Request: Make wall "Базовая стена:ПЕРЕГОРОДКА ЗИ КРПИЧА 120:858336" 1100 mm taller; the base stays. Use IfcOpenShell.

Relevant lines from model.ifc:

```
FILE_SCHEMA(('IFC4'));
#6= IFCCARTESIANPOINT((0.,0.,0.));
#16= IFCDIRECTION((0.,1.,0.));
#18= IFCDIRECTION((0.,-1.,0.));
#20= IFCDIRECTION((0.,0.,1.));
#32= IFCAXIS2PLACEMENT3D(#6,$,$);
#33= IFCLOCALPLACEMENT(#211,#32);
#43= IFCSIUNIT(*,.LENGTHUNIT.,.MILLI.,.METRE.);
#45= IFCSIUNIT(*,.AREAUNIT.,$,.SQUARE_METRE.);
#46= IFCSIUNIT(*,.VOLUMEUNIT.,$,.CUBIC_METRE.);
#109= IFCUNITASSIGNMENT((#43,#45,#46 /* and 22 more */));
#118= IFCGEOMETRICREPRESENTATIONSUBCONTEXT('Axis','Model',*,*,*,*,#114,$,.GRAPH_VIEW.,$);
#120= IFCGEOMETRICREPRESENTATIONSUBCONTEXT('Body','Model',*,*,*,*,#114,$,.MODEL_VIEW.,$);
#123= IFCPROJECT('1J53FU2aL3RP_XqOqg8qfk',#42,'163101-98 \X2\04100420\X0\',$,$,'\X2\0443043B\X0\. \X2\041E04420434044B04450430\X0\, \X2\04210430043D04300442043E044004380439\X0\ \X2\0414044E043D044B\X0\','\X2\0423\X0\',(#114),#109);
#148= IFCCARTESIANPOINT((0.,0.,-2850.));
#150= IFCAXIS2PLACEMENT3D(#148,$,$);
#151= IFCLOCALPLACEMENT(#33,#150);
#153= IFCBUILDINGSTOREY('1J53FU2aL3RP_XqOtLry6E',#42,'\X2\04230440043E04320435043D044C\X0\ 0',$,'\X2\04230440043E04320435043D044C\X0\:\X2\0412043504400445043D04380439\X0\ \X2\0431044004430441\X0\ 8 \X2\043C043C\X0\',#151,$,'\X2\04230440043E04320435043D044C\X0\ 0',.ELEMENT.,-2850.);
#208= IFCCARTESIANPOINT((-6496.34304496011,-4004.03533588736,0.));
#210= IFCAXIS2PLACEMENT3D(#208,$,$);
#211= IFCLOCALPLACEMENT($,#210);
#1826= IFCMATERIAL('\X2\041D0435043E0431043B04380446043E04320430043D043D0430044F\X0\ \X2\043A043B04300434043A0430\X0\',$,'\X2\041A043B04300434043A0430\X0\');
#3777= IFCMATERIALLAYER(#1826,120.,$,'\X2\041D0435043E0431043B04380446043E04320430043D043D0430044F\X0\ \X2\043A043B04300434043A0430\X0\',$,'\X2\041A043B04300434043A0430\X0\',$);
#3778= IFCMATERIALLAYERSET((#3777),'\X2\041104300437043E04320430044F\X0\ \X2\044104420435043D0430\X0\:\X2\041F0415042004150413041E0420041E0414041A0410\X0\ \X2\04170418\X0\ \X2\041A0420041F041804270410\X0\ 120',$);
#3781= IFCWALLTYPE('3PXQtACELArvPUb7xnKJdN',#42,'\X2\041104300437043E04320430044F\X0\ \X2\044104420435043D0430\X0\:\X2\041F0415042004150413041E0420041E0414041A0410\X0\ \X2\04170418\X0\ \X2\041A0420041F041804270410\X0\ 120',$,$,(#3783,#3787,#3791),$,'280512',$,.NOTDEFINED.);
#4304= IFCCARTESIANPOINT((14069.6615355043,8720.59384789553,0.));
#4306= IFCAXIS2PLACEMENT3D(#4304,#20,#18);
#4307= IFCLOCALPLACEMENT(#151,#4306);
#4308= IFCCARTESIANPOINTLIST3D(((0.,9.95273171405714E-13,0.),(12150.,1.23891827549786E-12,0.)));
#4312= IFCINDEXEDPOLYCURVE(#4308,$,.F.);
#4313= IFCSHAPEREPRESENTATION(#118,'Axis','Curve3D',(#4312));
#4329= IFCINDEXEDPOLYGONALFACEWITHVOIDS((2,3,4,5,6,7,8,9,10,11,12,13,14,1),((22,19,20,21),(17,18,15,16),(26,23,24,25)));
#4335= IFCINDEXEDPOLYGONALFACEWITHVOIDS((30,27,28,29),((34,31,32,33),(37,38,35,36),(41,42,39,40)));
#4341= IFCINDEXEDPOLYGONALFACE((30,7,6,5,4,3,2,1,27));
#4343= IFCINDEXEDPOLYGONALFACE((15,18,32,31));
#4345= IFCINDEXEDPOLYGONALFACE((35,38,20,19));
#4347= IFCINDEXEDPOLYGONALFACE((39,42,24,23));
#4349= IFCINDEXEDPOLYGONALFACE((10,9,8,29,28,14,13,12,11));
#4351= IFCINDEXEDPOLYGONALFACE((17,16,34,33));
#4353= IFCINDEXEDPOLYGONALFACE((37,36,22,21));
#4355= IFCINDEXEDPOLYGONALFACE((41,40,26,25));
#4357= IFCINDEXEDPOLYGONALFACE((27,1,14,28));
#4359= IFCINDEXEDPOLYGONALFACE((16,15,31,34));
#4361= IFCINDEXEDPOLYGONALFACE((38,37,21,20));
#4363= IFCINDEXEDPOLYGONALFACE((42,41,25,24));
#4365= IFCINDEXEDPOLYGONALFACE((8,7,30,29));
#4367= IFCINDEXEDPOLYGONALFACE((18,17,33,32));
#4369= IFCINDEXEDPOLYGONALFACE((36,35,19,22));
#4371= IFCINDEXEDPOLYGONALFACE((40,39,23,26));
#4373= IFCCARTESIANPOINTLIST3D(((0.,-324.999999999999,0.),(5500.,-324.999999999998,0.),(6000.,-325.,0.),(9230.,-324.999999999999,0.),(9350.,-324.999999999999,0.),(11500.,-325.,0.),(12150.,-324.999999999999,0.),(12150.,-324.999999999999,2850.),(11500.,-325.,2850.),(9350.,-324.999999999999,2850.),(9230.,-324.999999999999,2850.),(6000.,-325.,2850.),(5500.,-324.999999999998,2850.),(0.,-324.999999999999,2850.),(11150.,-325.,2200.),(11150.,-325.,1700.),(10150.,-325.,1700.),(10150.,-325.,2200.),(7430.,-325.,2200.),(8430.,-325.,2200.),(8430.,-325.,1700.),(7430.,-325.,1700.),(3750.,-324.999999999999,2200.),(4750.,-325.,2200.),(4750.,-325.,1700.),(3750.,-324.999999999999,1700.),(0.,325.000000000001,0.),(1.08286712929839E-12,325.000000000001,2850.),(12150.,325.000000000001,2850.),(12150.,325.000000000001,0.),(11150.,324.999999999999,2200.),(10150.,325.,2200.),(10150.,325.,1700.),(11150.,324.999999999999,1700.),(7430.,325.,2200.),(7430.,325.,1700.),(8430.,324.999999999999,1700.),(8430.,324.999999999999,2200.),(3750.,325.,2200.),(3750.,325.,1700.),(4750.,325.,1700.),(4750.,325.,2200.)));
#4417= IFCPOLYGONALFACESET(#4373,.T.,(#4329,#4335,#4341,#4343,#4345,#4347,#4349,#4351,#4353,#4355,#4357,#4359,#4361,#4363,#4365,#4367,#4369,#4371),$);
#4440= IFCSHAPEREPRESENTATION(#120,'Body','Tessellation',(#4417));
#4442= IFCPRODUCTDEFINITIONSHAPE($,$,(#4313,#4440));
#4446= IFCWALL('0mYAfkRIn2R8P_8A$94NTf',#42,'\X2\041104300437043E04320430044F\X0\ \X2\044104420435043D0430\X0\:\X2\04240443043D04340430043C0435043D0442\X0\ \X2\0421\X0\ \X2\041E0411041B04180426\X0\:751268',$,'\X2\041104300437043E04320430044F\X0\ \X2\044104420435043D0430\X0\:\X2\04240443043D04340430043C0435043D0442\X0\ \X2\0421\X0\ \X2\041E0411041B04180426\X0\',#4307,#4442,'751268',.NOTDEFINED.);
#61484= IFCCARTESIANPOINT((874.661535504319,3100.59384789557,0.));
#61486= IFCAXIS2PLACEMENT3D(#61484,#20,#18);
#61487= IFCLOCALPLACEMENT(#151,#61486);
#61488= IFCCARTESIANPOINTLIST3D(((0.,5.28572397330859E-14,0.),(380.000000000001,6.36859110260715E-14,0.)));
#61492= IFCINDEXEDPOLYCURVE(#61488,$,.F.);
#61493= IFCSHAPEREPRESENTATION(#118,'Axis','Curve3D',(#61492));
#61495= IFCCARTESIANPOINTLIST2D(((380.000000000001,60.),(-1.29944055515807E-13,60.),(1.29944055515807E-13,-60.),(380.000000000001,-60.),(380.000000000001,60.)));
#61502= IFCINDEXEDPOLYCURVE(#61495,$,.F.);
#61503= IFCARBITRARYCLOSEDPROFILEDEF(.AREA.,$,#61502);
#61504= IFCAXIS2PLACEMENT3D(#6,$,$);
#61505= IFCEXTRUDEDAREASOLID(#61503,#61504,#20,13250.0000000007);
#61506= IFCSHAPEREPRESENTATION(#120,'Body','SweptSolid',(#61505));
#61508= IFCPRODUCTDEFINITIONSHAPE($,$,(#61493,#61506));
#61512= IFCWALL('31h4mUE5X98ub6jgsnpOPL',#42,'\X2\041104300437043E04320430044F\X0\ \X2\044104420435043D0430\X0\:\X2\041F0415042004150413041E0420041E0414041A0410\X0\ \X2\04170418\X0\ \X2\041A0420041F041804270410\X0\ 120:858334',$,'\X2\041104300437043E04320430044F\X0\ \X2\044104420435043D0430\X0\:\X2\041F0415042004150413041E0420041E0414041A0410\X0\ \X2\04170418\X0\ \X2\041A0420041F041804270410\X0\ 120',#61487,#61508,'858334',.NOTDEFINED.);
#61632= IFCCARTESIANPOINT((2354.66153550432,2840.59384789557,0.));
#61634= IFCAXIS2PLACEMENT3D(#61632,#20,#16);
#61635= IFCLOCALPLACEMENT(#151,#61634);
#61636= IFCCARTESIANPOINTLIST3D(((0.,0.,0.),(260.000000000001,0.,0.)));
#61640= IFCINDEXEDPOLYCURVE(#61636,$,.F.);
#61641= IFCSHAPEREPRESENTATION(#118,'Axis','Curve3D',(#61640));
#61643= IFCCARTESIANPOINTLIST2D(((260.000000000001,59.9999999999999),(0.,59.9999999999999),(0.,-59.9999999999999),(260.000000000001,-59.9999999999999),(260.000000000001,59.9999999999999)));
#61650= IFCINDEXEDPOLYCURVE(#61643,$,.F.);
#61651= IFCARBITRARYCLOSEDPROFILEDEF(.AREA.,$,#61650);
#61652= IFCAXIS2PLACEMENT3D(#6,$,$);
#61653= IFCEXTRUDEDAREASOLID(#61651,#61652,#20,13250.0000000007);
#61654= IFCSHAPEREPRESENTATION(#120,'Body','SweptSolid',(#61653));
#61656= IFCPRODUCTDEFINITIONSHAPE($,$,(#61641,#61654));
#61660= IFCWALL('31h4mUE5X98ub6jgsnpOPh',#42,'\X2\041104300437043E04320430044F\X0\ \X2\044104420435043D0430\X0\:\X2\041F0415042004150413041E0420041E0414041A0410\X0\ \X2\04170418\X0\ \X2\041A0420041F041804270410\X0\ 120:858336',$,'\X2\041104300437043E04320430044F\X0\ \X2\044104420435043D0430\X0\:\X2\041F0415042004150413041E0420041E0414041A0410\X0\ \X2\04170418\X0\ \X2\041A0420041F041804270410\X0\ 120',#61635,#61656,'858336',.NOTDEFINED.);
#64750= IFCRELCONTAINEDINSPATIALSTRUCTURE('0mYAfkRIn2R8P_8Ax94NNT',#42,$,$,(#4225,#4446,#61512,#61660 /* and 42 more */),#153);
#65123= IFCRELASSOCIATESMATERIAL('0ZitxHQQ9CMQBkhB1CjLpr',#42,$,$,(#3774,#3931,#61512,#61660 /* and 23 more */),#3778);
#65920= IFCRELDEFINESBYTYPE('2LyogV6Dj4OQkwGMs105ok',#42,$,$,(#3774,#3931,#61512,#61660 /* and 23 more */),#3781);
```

```python
import ifcopenshell
import ifcopenshell.geom
import ifcopenshell.util.representation
import ifcopenshell.util.shape

model = ifcopenshell.open("model.ifc")
settings = ifcopenshell.geom.settings()


def volume(element):
    """Net volume in cubic metres, openings subtracted."""
    shape = ifcopenshell.geom.create_shape(settings, element)
    return ifcopenshell.util.shape.get_volume(shape.geometry)


wall = model.by_id(61660)
before = volume(wall)

body = ifcopenshell.util.representation.get_representation(wall, "Model", "Body")
solid = body.Items[0]
old_height = solid.Depth
solid.Depth += 1100.0
after = volume(wall)

print(f"height {old_height:g} -> {solid.Depth:g}, volume {before:.3f} -> {after:.3f} m3")

model.write("model-out.ifc")
```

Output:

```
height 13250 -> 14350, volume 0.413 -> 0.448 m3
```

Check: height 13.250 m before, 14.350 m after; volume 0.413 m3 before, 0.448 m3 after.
